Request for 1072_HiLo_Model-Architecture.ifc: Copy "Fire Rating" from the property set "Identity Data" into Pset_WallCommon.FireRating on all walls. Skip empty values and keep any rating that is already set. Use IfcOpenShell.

First a look at what the model holds.

```python
import ifcopenshell
import ifcopenshell.util.element

model = ifcopenshell.open("1072_HiLo_Model-Architecture.ifc")
print(model.schema)
walls = model.by_type("IfcWall")
print(len(walls), "walls")
for e in walls[:8]:
    source = ifcopenshell.util.element.get_pset(e, "Identity Data", "Fire Rating")
    target = ifcopenshell.util.element.get_pset(e, "Pset_WallCommon", "FireRating")
    print(e.id(), repr(source), repr(target), sep=" | ")
```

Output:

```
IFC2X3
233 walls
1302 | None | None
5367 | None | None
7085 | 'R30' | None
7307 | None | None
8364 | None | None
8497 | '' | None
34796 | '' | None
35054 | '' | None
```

```python
import ifcopenshell
import ifcopenshell.api.pset
import ifcopenshell.util.element

model = ifcopenshell.open("1072_HiLo_Model-Architecture.ifc")

count = 0
for e in model.by_type("IfcWall"):
    value = ifcopenshell.util.element.get_pset(e, "Identity Data", "Fire Rating")
    current = ifcopenshell.util.element.get_pset(e, "Pset_WallCommon", "FireRating")
    if not value or not value.strip() or current:
        continue
    # add_pset returns the element's existing set when there is one.
    pset = ifcopenshell.api.pset.add_pset(model, product=e, name="Pset_WallCommon")
    ifcopenshell.api.pset.edit_pset(model, pset=pset, properties={"FireRating": value})
    count += 1

print(count, "walls updated")

model.write("1072_HiLo_Model-Architecture-out.ifc")
```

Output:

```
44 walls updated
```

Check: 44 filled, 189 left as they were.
